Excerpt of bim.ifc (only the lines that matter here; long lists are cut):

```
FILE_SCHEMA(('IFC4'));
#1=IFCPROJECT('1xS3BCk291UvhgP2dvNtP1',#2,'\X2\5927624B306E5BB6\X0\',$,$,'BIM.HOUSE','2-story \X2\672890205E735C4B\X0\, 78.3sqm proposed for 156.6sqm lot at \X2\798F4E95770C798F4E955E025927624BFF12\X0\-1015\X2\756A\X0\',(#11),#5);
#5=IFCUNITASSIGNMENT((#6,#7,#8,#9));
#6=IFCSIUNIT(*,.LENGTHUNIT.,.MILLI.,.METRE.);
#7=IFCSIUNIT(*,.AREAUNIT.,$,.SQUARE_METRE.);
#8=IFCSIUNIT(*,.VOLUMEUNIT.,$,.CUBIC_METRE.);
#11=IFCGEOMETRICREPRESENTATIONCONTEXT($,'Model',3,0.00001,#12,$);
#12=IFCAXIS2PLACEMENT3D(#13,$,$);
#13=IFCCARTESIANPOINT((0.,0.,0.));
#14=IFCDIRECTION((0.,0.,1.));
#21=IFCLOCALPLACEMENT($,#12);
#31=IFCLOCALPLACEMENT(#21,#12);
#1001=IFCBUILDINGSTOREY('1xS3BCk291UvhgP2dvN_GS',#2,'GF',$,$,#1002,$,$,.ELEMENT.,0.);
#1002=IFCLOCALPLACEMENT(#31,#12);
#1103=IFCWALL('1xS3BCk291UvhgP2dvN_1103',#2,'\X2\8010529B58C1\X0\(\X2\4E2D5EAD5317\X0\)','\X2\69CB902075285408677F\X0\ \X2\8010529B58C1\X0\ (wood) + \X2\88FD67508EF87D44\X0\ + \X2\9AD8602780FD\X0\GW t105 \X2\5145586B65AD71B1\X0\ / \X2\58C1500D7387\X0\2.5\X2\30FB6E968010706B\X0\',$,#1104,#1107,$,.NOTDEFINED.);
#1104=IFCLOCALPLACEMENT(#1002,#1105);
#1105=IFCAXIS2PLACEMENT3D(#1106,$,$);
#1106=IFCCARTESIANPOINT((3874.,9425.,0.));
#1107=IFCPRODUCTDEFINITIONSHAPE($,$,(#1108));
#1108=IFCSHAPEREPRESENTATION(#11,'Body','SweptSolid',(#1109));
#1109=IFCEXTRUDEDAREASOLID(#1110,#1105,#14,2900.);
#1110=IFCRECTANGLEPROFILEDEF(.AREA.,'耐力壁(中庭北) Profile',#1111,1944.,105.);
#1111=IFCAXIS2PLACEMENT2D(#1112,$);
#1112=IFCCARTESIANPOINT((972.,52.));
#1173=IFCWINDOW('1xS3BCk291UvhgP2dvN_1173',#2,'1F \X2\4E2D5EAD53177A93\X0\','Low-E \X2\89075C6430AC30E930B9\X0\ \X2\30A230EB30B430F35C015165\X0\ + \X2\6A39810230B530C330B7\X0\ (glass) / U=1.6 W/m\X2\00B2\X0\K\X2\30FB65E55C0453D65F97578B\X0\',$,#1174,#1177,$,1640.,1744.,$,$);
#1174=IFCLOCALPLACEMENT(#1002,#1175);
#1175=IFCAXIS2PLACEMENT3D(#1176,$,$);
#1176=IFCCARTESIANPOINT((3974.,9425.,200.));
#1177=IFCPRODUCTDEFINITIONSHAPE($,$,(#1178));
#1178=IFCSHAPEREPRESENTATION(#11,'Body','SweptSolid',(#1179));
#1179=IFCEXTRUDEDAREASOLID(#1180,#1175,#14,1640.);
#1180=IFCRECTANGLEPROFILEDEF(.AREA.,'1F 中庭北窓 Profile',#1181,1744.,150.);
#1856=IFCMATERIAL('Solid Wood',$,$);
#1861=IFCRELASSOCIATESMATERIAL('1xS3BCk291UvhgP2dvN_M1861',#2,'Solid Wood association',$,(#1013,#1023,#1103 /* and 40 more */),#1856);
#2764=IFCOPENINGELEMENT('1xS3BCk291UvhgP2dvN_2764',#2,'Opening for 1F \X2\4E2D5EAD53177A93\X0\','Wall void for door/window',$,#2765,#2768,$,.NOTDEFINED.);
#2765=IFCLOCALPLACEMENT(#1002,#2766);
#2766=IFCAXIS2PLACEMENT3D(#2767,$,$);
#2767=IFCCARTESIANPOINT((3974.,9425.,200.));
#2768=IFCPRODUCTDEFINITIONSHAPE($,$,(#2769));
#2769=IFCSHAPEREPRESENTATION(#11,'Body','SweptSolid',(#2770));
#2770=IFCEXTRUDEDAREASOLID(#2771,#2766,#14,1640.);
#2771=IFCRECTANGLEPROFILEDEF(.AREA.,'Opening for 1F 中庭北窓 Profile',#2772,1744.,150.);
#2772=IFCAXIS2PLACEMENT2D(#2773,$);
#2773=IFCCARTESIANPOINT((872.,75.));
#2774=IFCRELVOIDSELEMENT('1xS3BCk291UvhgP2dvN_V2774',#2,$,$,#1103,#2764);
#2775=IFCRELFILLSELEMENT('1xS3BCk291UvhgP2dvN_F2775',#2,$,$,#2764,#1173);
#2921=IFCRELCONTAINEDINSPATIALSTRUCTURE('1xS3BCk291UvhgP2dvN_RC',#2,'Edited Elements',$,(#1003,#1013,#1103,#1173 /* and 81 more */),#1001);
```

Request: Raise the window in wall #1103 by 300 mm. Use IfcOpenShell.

```python
import numpy as np
import ifcopenshell
import ifcopenshell.api.geometry
import ifcopenshell.util.placement
import ifcopenshell.util.unit

model = ifcopenshell.open("bim.ifc")
unit_scale = ifcopenshell.util.unit.calculate_unit_scale(model)

window = model.by_guid("1xS3BCk291UvhgP2dvN_1173")
opening = window.FillsVoids[0].RelatingOpeningElement
dz = 0.3 / unit_scale

shift = np.array([0.0, 0.0, dz])
# The window is not placed relative to its opening, so move both.
for product in (opening, window):
    matrix = ifcopenshell.util.placement.get_local_placement(product.ObjectPlacement)
    matrix[:3, 3] += shift
    ifcopenshell.api.geometry.edit_object_placement(model, product=product, matrix=matrix, is_si=False)

print(f"moved by {dz * unit_scale:+.3f} m")

model.write("bim-out.ifc")
```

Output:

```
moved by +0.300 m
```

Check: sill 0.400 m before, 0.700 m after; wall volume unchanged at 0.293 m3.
